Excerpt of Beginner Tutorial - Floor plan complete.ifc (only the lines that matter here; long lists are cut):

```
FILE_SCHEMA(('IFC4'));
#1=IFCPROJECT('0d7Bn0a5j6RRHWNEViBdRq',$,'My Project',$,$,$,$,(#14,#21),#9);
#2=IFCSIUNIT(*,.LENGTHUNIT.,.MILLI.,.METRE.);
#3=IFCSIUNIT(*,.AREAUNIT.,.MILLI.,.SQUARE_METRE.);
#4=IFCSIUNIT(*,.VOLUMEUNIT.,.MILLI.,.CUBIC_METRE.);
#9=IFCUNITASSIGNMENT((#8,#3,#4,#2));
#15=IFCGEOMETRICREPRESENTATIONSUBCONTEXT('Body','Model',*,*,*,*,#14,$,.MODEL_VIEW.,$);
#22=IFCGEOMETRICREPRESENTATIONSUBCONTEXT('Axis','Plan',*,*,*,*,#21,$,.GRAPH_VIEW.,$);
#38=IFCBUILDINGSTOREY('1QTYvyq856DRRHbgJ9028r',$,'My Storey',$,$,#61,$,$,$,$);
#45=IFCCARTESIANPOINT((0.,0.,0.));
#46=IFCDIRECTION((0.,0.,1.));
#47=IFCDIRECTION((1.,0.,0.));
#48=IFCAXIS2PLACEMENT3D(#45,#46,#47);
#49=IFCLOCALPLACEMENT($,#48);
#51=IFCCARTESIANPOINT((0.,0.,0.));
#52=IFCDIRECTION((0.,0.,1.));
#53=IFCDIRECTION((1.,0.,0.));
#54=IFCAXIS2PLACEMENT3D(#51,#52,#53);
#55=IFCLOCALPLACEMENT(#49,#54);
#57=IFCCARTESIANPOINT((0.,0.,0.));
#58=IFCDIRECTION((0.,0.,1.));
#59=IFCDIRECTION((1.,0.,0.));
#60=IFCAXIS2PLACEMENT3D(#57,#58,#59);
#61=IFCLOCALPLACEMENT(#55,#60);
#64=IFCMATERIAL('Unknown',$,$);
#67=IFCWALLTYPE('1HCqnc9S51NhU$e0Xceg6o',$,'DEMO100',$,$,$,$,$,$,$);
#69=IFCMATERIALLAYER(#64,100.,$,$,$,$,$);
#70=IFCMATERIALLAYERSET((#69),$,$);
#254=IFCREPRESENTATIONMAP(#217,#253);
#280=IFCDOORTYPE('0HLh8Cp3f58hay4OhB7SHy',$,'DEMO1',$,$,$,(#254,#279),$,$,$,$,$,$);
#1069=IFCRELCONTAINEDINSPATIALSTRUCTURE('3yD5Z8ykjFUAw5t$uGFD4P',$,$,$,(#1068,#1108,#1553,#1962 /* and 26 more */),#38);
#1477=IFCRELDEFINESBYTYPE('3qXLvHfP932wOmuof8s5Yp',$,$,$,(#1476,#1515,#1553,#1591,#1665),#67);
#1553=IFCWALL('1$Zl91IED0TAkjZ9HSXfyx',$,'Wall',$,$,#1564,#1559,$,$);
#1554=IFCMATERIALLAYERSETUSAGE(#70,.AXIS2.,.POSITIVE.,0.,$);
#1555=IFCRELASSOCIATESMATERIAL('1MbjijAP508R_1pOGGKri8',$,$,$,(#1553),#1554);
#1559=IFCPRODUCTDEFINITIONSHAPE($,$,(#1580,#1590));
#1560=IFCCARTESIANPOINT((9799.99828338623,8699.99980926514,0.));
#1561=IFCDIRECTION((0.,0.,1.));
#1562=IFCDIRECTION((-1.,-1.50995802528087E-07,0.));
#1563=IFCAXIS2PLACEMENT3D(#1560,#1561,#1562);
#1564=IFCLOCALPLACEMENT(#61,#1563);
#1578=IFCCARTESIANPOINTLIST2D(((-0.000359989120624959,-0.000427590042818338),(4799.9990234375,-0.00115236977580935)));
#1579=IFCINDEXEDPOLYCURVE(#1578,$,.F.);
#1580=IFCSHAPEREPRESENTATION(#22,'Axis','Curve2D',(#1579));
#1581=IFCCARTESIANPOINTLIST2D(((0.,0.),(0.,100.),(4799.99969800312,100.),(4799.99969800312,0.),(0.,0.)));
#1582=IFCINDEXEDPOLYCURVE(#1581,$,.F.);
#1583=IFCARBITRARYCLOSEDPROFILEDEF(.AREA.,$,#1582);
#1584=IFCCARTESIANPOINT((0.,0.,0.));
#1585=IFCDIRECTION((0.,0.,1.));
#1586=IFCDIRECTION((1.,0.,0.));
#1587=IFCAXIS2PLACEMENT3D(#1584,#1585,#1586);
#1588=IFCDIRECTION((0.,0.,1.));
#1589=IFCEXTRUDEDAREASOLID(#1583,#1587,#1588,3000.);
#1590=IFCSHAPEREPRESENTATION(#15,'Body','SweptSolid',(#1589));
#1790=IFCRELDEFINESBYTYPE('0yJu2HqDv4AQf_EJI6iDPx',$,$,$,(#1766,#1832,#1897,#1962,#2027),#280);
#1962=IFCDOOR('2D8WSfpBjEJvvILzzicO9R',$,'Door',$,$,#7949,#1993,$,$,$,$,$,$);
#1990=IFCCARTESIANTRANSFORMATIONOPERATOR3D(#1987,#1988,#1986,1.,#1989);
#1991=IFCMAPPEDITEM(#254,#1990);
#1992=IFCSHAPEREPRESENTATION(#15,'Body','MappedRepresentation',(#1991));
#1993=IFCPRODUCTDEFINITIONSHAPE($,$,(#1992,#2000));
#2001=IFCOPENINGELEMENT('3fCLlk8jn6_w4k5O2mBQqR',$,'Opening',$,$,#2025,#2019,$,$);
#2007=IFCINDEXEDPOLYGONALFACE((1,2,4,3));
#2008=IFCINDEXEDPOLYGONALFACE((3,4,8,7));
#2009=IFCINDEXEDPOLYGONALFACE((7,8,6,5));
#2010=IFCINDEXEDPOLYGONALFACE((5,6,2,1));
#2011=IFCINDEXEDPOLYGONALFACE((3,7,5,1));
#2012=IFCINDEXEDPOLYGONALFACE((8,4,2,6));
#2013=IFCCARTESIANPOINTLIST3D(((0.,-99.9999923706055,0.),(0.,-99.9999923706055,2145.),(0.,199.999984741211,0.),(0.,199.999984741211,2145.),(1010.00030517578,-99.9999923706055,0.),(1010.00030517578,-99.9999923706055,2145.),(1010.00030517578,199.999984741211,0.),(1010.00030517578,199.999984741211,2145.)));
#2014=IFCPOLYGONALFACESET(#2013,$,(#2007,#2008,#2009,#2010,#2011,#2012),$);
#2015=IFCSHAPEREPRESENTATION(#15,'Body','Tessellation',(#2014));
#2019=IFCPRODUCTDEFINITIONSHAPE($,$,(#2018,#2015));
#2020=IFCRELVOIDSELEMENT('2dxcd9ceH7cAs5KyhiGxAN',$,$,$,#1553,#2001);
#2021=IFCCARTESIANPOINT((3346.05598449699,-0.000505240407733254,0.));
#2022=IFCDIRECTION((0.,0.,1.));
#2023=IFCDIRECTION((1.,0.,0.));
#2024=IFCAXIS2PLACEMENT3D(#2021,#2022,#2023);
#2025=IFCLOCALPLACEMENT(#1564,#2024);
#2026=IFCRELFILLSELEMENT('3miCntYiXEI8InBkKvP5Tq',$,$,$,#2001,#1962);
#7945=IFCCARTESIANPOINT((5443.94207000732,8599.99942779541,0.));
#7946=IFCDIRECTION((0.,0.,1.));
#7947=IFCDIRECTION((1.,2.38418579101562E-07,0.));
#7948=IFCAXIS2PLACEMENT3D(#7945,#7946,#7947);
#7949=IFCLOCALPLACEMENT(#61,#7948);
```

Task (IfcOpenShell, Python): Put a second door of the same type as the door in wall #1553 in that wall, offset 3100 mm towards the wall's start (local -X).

```python
import ifcopenshell
import ifcopenshell.api.feature
import ifcopenshell.api.geometry
import ifcopenshell.api.root
import ifcopenshell.geom
import ifcopenshell.util.element
import ifcopenshell.util.placement
import ifcopenshell.util.shape

model = ifcopenshell.open("Beginner Tutorial - Floor plan complete.ifc")
settings = ifcopenshell.geom.settings()


def volume(element):
    """Net volume in cubic metres, openings subtracted."""
    shape = ifcopenshell.geom.create_shape(settings, element)
    return ifcopenshell.util.shape.get_volume(shape.geometry)


door = model.by_guid("2D8WSfpBjEJvvILzzicO9R")
opening = door.FillsVoids[0].RelatingOpeningElement
wall = opening.VoidsElements[0].RelatingBuildingElement
before = volume(wall)
shift = ifcopenshell.util.placement.get_local_placement(wall.ObjectPlacement)[:3, 0] * -3100.0

# copy_class copies the void relationship, type, container and properties, but no geometry.
new_opening = ifcopenshell.api.root.copy_class(model, product=opening)
new_opening.Representation = ifcopenshell.util.element.copy_deep(
    model, opening.Representation, exclude=["IfcGeometricRepresentationContext", "IfcRepresentationMap"]
)
new_door = ifcopenshell.api.root.copy_class(model, product=door)
new_door.Representation = ifcopenshell.util.element.copy_deep(
    model, door.Representation, exclude=["IfcGeometricRepresentationContext", "IfcRepresentationMap"]
)
ifcopenshell.api.feature.add_filling(model, opening=new_opening, element=new_door)

for old, new in ((opening, new_opening), (door, new_door)):
    matrix = ifcopenshell.util.placement.get_local_placement(old.ObjectPlacement)
    matrix[:3, 3] += shift
    ifcopenshell.api.geometry.edit_object_placement(model, product=new, matrix=matrix, is_si=False)

after = volume(wall)

print(f"wall volume {before:.3f} -> {after:.3f} m3")

model.write("Beginner Tutorial - Floor plan complete_rev.ifc")
```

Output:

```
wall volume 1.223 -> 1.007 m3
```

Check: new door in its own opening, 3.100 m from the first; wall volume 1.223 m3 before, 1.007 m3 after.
